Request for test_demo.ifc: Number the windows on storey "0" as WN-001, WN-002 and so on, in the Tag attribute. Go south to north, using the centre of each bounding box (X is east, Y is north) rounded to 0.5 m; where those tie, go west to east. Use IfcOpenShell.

First a look at what the model holds.

```python
import ifcopenshell
import ifcopenshell.util.element
import ifcopenshell.util.placement

model = ifcopenshell.open("test_demo.ifc")
print(model.schema)
storey = next(s for s in model.by_type("IfcBuildingStorey") if s.Name == "0")
windows = [e for e in ifcopenshell.util.element.get_decomposition(storey) if e.is_a("IfcWindow")]
for e in sorted(windows, key=lambda e: e.id()):
    origin = ifcopenshell.util.placement.get_local_placement(e.ObjectPlacement)[:3, 3]
    print(e.id(), e.Tag, e.Name, origin.round(2) + 0.0, sep=" | ")
```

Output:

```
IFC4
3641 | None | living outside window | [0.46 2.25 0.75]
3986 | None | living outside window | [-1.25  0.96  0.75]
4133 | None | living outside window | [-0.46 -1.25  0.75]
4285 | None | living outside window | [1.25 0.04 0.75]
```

```python
import ifcopenshell
import ifcopenshell.geom
import ifcopenshell.util.element
import ifcopenshell.util.shape

model = ifcopenshell.open("test_demo.ifc")
settings = ifcopenshell.geom.settings()
settings.set("use-world-coords", True)


def centre(element):
    shape = ifcopenshell.geom.create_shape(settings, element)
    return ifcopenshell.util.shape.get_bbox_centroid(shape.geometry)


storey = next(s for s in model.by_type("IfcBuildingStorey") if s.Name == "0")
windows = [e for e in ifcopenshell.util.element.get_decomposition(storey) if e.is_a("IfcWindow")]

# Insertion points can sit at a corner or the storey origin, so sort by the geometry (in metres).
centres = {e: centre(e) for e in windows}
windows.sort(key=lambda e: (round(centres[e][1] / 0.5), centres[e][0]))

for i, e in enumerate(windows, start=1):
    number = f"WN-0{i:02d}"
    e.Tag = number
    print(e.id(), number)

model.write("test_demo_edited.ifc")
```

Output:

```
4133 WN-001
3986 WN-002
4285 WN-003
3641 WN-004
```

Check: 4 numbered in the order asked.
